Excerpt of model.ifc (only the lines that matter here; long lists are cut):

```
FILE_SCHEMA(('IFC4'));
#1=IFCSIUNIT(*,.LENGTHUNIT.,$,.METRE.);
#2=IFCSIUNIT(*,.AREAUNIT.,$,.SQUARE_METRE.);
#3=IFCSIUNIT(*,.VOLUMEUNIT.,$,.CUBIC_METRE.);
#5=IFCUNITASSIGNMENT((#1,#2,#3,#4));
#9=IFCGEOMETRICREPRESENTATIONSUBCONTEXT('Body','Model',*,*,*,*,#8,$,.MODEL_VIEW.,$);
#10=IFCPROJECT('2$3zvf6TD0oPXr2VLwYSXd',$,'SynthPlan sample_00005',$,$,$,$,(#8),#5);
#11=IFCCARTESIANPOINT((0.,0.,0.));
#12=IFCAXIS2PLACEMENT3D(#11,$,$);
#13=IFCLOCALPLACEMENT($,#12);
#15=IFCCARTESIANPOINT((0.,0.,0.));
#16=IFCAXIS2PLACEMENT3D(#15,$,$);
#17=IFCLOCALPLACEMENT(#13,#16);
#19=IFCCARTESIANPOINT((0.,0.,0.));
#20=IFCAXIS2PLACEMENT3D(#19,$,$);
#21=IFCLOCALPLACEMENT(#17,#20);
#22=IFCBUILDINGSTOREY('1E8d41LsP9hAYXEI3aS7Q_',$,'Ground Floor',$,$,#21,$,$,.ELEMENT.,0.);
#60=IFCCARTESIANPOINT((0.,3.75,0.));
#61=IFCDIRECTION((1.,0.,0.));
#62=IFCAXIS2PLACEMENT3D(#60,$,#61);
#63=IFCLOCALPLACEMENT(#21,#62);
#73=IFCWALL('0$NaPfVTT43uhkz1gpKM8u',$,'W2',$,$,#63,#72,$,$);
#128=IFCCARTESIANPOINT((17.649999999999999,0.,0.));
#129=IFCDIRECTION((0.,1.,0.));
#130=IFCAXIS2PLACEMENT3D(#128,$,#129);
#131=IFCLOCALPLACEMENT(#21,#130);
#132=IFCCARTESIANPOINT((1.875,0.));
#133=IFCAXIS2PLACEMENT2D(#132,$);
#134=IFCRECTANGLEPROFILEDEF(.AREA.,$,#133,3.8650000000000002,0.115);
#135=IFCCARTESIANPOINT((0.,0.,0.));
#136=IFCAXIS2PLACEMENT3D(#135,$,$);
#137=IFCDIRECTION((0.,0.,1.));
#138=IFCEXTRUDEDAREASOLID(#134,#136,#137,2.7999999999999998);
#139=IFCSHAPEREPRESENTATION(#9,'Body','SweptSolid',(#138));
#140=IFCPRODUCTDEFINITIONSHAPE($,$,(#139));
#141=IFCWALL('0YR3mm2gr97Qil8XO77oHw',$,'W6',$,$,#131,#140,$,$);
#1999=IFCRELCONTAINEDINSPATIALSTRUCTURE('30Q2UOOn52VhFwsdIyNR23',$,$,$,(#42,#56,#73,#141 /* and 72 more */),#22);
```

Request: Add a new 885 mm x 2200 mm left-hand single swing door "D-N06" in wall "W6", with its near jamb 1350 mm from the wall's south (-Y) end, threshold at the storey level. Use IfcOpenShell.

```python
import numpy as np
import ifcopenshell
import ifcopenshell.api.feature
import ifcopenshell.api.geometry
import ifcopenshell.api.root
import ifcopenshell.api.spatial
import ifcopenshell.geom
import ifcopenshell.util.element
import ifcopenshell.util.placement
import ifcopenshell.util.representation
import ifcopenshell.util.shape
import ifcopenshell.util.unit

model = ifcopenshell.open("model.ifc")
unit_scale = ifcopenshell.util.unit.calculate_unit_scale(model)
settings = ifcopenshell.geom.settings()


def volume(element):
    """Net volume in cubic metres, openings subtracted."""
    shape = ifcopenshell.geom.create_shape(settings, element)
    return ifcopenshell.util.shape.get_volume(shape.geometry)


wall = model.by_guid("0YR3mm2gr97Qil8XO77oHw")
storey = ifcopenshell.util.element.get_container(wall, ifc_class="IfcBuildingStorey")
context = ifcopenshell.util.representation.get_context(model, "Model", "Body", "MODEL_VIEW")
before = volume(wall)

width, height, from_end, sill = 0.885, 2.2, 1.35, 0.0  # metres

# The wall runs along its own X axis, and the end named is its -X end.
wall_shape = ifcopenshell.geom.create_shape(settings, wall)
x, y, z = ifcopenshell.util.shape.get_vertices(wall_shape.geometry).T
start = x.min() + from_end
face, thickness = float(y.min()), float(y.max() - y.min())
wall_matrix = ifcopenshell.util.placement.get_local_placement(wall.ObjectPlacement)
level = ifcopenshell.util.placement.get_local_placement(storey.ObjectPlacement)[2, 3]


def in_wall(x, y):
    """Placement at x, y metres in the wall's axes, at sill height."""
    matrix = wall_matrix.copy()
    matrix[:, 3] = wall_matrix @ np.array([x / unit_scale, y / unit_scale, 0.0, 1.0])
    matrix[2, 3] = level + sill / unit_scale
    return matrix


# Opening: a box that overshoots both wall faces by 50 mm.
opening = ifcopenshell.api.root.create_entity(model, ifc_class="IfcOpeningElement", predefined_type="OPENING")
box = ifcopenshell.api.geometry.add_wall_representation(
    model, context=context, length=width, height=height, thickness=thickness + 0.1
)
ifcopenshell.api.geometry.assign_representation(model, product=opening, representation=box)
ifcopenshell.api.geometry.edit_object_placement(model, product=opening, matrix=in_wall(start, face - 0.05), is_si=False)
ifcopenshell.api.feature.add_feature(model, feature=opening, element=wall)

door = ifcopenshell.api.root.create_entity(model, ifc_class="IfcDoor", name="D-N06", predefined_type="DOOR")
door.OverallWidth, door.OverallHeight = width / unit_scale, height / unit_scale
door.OperationType = "SINGLE_SWING_LEFT"
body = ifcopenshell.api.geometry.add_door_representation(
    model,
    context=context,
    overall_width=door.OverallWidth,
    overall_height=door.OverallHeight,
    operation_type="SINGLE_SWING_LEFT",
    lining_properties={"LiningDepth": thickness / unit_scale, "ThresholdDepth": thickness / unit_scale},
)
ifcopenshell.api.geometry.assign_representation(model, product=door, representation=body)
ifcopenshell.api.spatial.assign_container(model, products=[door], relating_structure=storey)
ifcopenshell.api.feature.add_filling(model, opening=opening, element=door)

# The lining spans the wall, so the door starts at the wall face.
ifcopenshell.api.geometry.edit_object_placement(model, product=door, matrix=in_wall(start, face), is_si=False)

after = volume(wall)

print(f"wall volume {before:.3f} -> {after:.3f} m3")

model.write("model_v2.ifc")
```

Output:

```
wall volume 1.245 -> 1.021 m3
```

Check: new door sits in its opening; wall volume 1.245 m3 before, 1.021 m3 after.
